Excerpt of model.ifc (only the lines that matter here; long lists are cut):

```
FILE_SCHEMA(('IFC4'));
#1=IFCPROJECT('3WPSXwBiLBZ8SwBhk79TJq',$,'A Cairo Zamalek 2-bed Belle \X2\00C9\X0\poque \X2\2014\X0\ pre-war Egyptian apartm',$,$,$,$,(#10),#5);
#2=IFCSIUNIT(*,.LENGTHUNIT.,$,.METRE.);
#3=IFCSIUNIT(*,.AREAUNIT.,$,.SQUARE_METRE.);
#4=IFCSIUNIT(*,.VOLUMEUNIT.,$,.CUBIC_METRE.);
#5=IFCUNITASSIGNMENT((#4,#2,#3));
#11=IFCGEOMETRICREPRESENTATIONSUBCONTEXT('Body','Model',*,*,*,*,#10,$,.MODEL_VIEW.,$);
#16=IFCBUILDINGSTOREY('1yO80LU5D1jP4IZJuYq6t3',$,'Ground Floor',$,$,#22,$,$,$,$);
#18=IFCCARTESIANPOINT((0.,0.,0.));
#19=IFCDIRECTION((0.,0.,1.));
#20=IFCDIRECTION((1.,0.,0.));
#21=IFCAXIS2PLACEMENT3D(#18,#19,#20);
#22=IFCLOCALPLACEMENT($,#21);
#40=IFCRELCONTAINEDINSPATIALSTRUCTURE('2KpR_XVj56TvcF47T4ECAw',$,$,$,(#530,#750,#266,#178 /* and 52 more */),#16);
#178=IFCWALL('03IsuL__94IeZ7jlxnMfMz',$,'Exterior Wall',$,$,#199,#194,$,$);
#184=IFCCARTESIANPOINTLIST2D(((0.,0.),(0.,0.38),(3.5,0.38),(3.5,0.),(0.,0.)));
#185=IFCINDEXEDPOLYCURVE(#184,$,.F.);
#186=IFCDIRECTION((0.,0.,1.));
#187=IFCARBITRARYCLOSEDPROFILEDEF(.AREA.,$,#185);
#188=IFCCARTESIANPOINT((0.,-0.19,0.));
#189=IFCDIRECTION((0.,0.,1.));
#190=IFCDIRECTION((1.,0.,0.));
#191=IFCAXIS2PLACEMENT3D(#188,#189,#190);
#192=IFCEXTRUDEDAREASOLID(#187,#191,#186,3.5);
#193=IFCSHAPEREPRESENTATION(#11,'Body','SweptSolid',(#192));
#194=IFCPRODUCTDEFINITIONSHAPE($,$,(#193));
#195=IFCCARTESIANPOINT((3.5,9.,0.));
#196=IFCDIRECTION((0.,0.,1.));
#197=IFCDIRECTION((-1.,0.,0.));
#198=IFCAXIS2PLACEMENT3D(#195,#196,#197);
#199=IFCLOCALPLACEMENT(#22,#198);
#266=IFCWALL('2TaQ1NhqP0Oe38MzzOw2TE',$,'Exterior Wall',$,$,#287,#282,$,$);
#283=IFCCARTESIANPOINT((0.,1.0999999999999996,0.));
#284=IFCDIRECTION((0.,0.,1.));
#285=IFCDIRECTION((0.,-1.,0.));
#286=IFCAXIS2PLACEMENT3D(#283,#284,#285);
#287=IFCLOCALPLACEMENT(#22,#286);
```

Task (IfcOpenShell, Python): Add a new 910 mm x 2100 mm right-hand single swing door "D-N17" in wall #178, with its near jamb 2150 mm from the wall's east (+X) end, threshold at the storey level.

```python
import numpy as np
import ifcopenshell
import ifcopenshell.api.feature
import ifcopenshell.api.geometry
import ifcopenshell.api.root
import ifcopenshell.api.spatial
import ifcopenshell.geom
import ifcopenshell.util.element
import ifcopenshell.util.placement
import ifcopenshell.util.representation
import ifcopenshell.util.shape
import ifcopenshell.util.unit

model = ifcopenshell.open("model.ifc")
unit_scale = ifcopenshell.util.unit.calculate_unit_scale(model)
settings = ifcopenshell.geom.settings()


def volume(element):
    """Net volume in cubic metres, openings subtracted."""
    shape = ifcopenshell.geom.create_shape(settings, element)
    return ifcopenshell.util.shape.get_volume(shape.geometry)


wall = model.by_guid("03IsuL__94IeZ7jlxnMfMz")
storey = ifcopenshell.util.element.get_container(wall, ifc_class="IfcBuildingStorey")
context = ifcopenshell.util.representation.get_context(model, "Model", "Body", "MODEL_VIEW")
before = volume(wall)

width, height, from_end, sill = 0.91, 2.1, 2.15, 0.0  # metres

# The wall runs along its own X axis, and the end named is its -X end.
wall_shape = ifcopenshell.geom.create_shape(settings, wall)
x, y, z = ifcopenshell.util.shape.get_vertices(wall_shape.geometry).T
start = x.min() + from_end
face, thickness = float(y.min()), float(y.max() - y.min())
wall_matrix = ifcopenshell.util.placement.get_local_placement(wall.ObjectPlacement)
level = ifcopenshell.util.placement.get_local_placement(storey.ObjectPlacement)[2, 3]


def in_wall(x, y):
    """Placement at x, y metres in the wall's axes, at sill height."""
    matrix = wall_matrix.copy()
    matrix[:, 3] = wall_matrix @ np.array([x / unit_scale, y / unit_scale, 0.0, 1.0])
    matrix[2, 3] = level + sill / unit_scale
    return matrix


# Opening: a box that overshoots both wall faces by 50 mm.
opening = ifcopenshell.api.root.create_entity(model, ifc_class="IfcOpeningElement", predefined_type="OPENING")
box = ifcopenshell.api.geometry.add_wall_representation(
    model, context=context, length=width, height=height, thickness=thickness + 0.1
)
ifcopenshell.api.geometry.assign_representation(model, product=opening, representation=box)
ifcopenshell.api.geometry.edit_object_placement(model, product=opening, matrix=in_wall(start, face - 0.05), is_si=False)
ifcopenshell.api.feature.add_feature(model, feature=opening, element=wall)

door = ifcopenshell.api.root.create_entity(model, ifc_class="IfcDoor", name="D-N17", predefined_type="DOOR")
door.OverallWidth, door.OverallHeight = width / unit_scale, height / unit_scale
door.OperationType = "SINGLE_SWING_RIGHT"
body = ifcopenshell.api.geometry.add_door_representation(
    model,
    context=context,
    overall_width=door.OverallWidth,
    overall_height=door.OverallHeight,
    operation_type="SINGLE_SWING_RIGHT",
    lining_properties={"LiningDepth": thickness / unit_scale, "ThresholdDepth": thickness / unit_scale},
)
ifcopenshell.api.geometry.assign_representation(model, product=door, representation=body)
ifcopenshell.api.spatial.assign_container(model, products=[door], relating_structure=storey)
ifcopenshell.api.feature.add_filling(model, opening=opening, element=door)

# The lining spans the wall, so the door starts at the wall face.
ifcopenshell.api.geometry.edit_object_placement(model, product=door, matrix=in_wall(start, face), is_si=False)

after = volume(wall)

print(f"wall volume {before:.3f} -> {after:.3f} m3")

model.write("model_v2.ifc")
```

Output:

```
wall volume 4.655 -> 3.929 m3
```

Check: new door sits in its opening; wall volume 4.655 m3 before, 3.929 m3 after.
